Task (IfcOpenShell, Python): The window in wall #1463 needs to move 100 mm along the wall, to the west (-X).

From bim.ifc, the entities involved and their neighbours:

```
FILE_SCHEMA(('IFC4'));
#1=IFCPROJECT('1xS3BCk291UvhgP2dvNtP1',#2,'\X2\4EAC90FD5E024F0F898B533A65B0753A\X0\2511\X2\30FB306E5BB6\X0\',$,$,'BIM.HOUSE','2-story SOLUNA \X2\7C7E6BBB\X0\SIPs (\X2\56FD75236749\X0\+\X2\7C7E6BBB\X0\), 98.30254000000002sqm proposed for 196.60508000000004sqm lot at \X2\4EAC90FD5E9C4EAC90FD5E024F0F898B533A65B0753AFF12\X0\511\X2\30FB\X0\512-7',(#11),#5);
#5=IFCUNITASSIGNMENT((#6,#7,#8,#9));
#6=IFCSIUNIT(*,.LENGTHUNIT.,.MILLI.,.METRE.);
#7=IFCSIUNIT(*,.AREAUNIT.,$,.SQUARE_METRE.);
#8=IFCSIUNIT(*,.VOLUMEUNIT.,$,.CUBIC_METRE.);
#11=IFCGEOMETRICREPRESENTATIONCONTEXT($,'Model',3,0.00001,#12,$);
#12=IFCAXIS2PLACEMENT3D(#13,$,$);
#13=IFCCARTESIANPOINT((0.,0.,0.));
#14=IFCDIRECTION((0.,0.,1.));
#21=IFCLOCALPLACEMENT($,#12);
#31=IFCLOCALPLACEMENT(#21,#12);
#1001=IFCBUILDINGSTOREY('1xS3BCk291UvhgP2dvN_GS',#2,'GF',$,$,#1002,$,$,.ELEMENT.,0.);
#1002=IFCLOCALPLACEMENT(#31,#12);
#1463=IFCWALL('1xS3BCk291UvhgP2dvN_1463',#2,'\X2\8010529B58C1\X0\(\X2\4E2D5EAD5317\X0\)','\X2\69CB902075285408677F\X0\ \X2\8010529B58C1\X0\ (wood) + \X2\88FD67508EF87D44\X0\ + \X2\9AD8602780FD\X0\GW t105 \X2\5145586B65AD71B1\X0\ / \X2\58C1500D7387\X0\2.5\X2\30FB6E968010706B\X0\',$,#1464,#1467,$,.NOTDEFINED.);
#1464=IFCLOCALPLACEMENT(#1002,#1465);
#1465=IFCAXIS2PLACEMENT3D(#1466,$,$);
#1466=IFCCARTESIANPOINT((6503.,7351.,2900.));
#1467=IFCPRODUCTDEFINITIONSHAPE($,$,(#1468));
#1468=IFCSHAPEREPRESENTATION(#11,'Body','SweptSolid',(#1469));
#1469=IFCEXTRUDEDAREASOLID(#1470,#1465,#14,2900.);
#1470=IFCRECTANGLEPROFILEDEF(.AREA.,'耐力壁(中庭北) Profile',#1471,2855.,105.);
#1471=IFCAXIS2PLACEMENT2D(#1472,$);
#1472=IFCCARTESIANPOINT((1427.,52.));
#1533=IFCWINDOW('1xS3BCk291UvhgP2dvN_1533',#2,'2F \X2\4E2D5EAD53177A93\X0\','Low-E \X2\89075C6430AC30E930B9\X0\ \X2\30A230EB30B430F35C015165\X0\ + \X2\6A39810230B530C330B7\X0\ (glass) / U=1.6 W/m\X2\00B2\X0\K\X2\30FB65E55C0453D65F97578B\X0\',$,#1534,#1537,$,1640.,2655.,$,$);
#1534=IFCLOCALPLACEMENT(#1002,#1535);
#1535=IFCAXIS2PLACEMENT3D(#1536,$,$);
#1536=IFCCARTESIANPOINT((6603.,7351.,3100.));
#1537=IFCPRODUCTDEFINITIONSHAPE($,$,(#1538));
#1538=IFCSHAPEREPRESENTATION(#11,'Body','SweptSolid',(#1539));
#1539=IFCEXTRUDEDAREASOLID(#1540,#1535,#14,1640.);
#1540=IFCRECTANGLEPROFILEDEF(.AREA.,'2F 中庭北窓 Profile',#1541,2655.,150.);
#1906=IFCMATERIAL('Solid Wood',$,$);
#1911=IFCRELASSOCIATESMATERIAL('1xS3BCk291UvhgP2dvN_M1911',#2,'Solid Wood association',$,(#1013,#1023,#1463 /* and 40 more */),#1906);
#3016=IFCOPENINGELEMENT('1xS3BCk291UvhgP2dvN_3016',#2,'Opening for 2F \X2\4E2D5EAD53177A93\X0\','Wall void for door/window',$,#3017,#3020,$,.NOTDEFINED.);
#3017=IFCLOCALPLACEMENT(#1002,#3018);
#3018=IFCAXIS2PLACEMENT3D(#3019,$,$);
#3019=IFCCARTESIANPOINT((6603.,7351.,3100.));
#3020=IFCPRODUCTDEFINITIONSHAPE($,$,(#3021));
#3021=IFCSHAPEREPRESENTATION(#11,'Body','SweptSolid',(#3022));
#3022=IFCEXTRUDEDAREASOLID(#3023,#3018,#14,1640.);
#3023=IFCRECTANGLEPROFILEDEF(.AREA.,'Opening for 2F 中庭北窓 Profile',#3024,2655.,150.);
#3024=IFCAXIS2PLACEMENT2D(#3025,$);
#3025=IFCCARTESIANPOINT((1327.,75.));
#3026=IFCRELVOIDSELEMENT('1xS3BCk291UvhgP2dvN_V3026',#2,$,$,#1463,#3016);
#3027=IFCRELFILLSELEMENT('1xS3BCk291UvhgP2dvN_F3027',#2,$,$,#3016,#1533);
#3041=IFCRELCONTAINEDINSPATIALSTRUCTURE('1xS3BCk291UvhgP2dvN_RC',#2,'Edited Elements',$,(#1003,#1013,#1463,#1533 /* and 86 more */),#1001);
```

```python
import ifcopenshell
import ifcopenshell.api.geometry
import ifcopenshell.util.placement
import ifcopenshell.util.unit

model = ifcopenshell.open("bim.ifc")
unit_scale = ifcopenshell.util.unit.calculate_unit_scale(model)

window = model.by_id(1533)
opening = window.FillsVoids[0].RelatingOpeningElement
wall = opening.VoidsElements[0].RelatingBuildingElement

wall_matrix = ifcopenshell.util.placement.get_local_placement(wall.ObjectPlacement)
shift = wall_matrix[:3, 0] * -0.1 / unit_scale
before = ifcopenshell.util.placement.get_local_placement(window.ObjectPlacement)[:3, 3].copy()

# The window is not placed relative to its opening, so move both.
for product in (opening, window):
    matrix = ifcopenshell.util.placement.get_local_placement(product.ObjectPlacement)
    matrix[:3, 3] += shift
    ifcopenshell.api.geometry.edit_object_placement(model, product=product, matrix=matrix, is_si=False)

after = ifcopenshell.util.placement.get_local_placement(window.ObjectPlacement)[:3, 3]
print("window moved by", (after - before).round(3) + 0.0)

model.write("bim_rev.ifc")
```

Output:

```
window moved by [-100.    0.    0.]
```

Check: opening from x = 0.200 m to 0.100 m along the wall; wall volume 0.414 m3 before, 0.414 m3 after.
